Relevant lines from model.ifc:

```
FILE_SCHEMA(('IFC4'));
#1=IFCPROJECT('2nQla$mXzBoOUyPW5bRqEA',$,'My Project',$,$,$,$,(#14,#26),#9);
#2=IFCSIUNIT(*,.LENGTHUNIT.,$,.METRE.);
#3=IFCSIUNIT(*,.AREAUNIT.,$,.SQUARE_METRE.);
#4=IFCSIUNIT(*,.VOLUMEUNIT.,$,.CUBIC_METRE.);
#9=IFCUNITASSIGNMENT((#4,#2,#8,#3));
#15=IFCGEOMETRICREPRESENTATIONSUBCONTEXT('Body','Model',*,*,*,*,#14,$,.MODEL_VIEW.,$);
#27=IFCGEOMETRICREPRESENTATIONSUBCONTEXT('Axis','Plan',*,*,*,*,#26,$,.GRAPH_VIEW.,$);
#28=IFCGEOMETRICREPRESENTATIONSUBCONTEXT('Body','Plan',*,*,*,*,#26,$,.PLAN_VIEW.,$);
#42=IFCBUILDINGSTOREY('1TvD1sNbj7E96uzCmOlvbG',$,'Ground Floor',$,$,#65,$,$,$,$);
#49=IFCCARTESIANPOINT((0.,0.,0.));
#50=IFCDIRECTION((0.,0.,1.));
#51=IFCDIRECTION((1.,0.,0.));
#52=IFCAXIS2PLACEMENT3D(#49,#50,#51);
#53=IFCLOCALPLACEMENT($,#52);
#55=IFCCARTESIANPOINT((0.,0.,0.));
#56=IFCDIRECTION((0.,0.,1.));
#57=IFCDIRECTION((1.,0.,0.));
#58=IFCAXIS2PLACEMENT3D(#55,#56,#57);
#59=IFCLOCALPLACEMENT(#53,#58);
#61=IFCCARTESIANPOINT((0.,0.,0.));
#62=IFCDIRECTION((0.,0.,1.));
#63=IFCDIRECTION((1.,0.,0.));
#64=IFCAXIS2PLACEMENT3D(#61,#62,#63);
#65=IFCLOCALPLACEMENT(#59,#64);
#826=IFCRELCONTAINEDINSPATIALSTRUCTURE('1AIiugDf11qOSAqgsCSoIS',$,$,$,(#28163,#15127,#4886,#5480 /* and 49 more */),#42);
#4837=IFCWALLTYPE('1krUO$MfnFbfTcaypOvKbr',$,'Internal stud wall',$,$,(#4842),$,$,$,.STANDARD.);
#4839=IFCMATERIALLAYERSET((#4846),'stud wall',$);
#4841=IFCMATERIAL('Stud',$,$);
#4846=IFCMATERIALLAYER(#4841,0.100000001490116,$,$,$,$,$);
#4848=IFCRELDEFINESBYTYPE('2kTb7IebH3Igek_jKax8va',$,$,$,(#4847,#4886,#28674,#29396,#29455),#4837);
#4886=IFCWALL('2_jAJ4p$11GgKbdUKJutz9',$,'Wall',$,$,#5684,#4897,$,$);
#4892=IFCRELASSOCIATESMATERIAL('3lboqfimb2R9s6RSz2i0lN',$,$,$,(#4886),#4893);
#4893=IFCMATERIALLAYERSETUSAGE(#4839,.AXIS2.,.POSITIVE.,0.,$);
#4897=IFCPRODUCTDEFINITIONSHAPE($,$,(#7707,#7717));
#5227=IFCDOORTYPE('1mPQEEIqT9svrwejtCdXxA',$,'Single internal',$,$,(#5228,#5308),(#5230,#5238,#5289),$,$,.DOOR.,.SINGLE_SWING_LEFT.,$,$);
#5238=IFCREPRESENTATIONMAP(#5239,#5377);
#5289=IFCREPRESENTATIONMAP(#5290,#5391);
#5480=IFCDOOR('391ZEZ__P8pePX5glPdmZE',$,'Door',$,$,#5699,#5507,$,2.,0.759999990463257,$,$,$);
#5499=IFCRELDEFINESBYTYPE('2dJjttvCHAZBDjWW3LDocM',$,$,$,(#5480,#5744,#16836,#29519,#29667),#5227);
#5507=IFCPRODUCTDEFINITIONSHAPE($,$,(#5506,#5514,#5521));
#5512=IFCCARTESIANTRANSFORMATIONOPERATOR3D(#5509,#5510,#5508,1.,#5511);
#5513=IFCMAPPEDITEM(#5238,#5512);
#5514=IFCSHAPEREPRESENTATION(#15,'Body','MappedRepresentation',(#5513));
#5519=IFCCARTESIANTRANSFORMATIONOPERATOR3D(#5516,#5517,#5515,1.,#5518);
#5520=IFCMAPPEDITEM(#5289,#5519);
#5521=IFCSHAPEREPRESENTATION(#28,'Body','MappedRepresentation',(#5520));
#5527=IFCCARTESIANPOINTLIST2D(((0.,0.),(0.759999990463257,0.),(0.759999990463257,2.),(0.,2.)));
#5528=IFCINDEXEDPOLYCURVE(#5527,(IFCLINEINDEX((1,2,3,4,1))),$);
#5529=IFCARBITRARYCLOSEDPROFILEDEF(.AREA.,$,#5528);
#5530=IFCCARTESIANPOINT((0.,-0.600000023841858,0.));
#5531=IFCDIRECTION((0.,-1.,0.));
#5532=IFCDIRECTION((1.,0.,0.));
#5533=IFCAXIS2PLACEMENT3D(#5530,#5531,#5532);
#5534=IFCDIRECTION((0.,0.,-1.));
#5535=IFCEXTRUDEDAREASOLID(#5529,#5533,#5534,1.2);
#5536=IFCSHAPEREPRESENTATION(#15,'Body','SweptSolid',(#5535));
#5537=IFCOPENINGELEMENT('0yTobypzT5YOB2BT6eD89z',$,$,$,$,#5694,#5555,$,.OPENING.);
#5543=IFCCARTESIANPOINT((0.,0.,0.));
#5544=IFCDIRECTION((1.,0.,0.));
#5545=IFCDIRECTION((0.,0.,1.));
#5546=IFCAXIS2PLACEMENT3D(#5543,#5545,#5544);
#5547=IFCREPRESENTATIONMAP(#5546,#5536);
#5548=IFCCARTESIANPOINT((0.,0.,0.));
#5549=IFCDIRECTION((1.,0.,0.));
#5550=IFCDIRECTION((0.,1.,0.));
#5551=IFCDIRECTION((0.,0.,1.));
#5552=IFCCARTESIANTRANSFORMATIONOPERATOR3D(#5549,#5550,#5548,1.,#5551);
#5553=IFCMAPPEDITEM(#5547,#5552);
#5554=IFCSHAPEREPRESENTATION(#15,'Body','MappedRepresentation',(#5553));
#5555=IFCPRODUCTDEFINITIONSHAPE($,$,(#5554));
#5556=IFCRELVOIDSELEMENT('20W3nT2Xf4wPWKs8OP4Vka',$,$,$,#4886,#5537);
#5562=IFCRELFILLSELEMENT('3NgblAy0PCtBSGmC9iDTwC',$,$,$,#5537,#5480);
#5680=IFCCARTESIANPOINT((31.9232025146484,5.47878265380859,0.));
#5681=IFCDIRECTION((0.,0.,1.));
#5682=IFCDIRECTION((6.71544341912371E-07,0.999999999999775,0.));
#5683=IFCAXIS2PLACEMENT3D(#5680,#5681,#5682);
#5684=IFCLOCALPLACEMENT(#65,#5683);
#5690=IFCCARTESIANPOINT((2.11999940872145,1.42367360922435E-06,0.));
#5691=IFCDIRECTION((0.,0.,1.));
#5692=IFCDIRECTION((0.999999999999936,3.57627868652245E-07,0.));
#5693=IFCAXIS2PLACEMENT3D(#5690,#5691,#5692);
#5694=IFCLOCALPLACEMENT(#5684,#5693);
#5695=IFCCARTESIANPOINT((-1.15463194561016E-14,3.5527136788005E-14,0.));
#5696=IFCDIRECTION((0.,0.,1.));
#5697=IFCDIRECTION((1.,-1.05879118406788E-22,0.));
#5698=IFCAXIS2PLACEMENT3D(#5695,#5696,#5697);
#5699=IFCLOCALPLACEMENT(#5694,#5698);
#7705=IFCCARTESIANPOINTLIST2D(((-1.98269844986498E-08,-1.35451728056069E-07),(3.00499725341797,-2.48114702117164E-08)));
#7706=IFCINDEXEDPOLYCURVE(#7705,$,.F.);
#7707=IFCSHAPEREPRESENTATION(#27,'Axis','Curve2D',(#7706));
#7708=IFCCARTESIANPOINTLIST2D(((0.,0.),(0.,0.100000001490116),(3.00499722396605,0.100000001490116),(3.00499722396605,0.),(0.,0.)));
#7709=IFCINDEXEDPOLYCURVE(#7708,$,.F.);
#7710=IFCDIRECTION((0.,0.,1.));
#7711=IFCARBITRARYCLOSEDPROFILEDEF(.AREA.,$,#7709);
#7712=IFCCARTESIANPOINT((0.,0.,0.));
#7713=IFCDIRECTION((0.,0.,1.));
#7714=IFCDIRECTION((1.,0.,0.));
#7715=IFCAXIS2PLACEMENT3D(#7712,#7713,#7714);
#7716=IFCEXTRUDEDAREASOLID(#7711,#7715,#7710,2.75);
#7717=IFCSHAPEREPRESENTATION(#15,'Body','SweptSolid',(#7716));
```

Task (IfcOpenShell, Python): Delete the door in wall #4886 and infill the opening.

```python
import ifcopenshell
import ifcopenshell.api.feature
import ifcopenshell.api.root
import ifcopenshell.geom
import ifcopenshell.util.shape

model = ifcopenshell.open("model.ifc")
settings = ifcopenshell.geom.settings()


def volume(element):
    """Net volume in cubic metres, openings subtracted."""
    shape = ifcopenshell.geom.create_shape(settings, element)
    return ifcopenshell.util.shape.get_volume(shape.geometry)


door = model.by_guid("391ZEZ__P8pePX5glPdmZE")
opening = door.FillsVoids[0].RelatingOpeningElement
wall = opening.VoidsElements[0].RelatingBuildingElement
before = volume(wall)

ifcopenshell.api.root.remove_product(model, product=door)
ifcopenshell.api.feature.remove_feature(model, feature=opening)

after = volume(wall)

print(f"wall volume {before:.3f} -> {after:.3f} m3")

model.write("model_rev.ifc")
```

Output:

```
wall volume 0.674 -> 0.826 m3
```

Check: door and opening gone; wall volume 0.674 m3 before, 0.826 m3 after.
